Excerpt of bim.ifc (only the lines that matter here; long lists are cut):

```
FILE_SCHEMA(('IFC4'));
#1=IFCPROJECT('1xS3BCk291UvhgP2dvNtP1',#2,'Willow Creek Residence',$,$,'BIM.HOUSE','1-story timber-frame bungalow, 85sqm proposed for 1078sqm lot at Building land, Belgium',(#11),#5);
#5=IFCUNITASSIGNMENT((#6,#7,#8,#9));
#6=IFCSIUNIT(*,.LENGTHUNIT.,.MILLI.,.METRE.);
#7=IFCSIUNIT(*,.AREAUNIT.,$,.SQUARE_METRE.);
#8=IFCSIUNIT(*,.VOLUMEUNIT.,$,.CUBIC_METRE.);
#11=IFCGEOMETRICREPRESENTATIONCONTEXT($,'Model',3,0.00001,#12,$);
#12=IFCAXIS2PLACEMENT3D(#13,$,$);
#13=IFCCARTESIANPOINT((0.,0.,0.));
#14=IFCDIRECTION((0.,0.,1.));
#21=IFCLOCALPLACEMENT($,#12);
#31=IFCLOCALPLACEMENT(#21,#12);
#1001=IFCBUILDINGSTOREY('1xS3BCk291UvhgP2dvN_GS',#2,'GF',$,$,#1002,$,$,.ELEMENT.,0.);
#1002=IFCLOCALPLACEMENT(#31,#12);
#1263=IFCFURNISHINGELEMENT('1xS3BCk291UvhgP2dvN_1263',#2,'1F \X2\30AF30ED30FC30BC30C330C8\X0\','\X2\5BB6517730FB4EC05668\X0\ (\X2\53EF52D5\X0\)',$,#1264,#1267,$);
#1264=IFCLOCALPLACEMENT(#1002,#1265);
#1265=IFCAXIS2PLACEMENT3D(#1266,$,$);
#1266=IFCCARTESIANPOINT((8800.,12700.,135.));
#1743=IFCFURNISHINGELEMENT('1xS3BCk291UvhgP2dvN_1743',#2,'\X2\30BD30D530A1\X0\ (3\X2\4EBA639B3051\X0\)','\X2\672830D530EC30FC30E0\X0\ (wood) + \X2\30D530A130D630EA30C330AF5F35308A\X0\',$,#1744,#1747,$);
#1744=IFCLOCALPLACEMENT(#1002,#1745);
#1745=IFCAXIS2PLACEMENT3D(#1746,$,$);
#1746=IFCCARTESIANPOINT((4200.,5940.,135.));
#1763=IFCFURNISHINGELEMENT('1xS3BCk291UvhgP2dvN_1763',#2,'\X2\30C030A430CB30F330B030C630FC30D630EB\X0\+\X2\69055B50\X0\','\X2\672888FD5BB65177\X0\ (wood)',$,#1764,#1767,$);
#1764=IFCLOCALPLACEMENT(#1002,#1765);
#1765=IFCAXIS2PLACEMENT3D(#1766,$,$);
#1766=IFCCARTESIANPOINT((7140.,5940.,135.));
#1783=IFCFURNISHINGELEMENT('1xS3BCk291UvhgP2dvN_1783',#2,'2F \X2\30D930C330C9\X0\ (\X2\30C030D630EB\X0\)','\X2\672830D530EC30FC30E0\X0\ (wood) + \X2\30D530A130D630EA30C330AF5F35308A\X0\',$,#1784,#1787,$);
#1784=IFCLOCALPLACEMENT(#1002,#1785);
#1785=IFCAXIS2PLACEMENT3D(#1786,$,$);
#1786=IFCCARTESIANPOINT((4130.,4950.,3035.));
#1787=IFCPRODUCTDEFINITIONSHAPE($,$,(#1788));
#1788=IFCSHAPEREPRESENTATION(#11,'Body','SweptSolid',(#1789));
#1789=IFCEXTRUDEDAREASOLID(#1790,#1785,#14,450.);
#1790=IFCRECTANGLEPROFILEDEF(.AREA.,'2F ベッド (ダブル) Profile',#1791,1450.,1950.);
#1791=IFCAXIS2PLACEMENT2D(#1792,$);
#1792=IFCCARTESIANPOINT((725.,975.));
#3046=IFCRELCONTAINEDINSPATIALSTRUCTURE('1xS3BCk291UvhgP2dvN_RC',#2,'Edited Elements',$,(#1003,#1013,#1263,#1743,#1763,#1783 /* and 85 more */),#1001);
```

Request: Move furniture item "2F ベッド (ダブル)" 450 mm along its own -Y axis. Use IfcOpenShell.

```python
import ifcopenshell
import ifcopenshell.api.geometry
import ifcopenshell.util.placement
import ifcopenshell.util.unit

model = ifcopenshell.open("bim.ifc")
unit_scale = ifcopenshell.util.unit.calculate_unit_scale(model)

item = model.by_guid("1xS3BCk291UvhgP2dvN_1783")
matrix = ifcopenshell.util.placement.get_local_placement(item.ObjectPlacement)
matrix[:3, 3] -= matrix[:3, 1] * 0.45 / unit_scale
ifcopenshell.api.geometry.edit_object_placement(model, product=item, matrix=matrix, is_si=False)

print(ifcopenshell.util.placement.get_local_placement(item.ObjectPlacement).round(3) + 0.0)

model.write("bim_rev.ifc")
```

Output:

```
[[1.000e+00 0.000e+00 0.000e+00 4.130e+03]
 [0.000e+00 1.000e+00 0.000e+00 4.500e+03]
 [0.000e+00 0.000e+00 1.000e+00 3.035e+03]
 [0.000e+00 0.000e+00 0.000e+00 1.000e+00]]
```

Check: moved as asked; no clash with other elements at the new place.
